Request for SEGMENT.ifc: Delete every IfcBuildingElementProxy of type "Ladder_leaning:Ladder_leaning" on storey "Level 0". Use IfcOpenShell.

First a look at what the model holds.

```python
import ifcopenshell
import ifcopenshell.util.element

model = ifcopenshell.open("SEGMENT.ifc")
print(model.schema)
storey = next(s for s in model.by_type("IfcBuildingStorey") if s.Name == "Level 0")
proxies = [e for e in ifcopenshell.util.element.get_decomposition(storey) if e.is_a("IfcBuildingElementProxy")]
seen = {}
for e in proxies:
    element_type = ifcopenshell.util.element.get_type(e)
    name = element_type.Name if element_type not in (None, e) else None
    seen[name] = seen.get(name, 0) + 1
for name, count in sorted(seen.items(), key=str):
    print(count, "x", name)
```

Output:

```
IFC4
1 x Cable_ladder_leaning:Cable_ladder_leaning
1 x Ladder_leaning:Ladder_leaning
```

```python
import ifcopenshell
import ifcopenshell.api.root
import ifcopenshell.util.element

model = ifcopenshell.open("SEGMENT.ifc")

storey = next(s for s in model.by_type("IfcBuildingStorey") if s.Name == "Level 0")
proxies = [e for e in ifcopenshell.util.element.get_decomposition(storey) if e.is_a("IfcBuildingElementProxy")]
targets = [e for e in proxies if (t := ifcopenshell.util.element.get_type(e)) not in (None, e) and t.Name == "Ladder_leaning:Ladder_leaning"]

for e in targets:
    ifcopenshell.api.root.remove_product(model, product=e)
print(len(targets), "removed")

model.write("SEGMENT_rev.ifc")
```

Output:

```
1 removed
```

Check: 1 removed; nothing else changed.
